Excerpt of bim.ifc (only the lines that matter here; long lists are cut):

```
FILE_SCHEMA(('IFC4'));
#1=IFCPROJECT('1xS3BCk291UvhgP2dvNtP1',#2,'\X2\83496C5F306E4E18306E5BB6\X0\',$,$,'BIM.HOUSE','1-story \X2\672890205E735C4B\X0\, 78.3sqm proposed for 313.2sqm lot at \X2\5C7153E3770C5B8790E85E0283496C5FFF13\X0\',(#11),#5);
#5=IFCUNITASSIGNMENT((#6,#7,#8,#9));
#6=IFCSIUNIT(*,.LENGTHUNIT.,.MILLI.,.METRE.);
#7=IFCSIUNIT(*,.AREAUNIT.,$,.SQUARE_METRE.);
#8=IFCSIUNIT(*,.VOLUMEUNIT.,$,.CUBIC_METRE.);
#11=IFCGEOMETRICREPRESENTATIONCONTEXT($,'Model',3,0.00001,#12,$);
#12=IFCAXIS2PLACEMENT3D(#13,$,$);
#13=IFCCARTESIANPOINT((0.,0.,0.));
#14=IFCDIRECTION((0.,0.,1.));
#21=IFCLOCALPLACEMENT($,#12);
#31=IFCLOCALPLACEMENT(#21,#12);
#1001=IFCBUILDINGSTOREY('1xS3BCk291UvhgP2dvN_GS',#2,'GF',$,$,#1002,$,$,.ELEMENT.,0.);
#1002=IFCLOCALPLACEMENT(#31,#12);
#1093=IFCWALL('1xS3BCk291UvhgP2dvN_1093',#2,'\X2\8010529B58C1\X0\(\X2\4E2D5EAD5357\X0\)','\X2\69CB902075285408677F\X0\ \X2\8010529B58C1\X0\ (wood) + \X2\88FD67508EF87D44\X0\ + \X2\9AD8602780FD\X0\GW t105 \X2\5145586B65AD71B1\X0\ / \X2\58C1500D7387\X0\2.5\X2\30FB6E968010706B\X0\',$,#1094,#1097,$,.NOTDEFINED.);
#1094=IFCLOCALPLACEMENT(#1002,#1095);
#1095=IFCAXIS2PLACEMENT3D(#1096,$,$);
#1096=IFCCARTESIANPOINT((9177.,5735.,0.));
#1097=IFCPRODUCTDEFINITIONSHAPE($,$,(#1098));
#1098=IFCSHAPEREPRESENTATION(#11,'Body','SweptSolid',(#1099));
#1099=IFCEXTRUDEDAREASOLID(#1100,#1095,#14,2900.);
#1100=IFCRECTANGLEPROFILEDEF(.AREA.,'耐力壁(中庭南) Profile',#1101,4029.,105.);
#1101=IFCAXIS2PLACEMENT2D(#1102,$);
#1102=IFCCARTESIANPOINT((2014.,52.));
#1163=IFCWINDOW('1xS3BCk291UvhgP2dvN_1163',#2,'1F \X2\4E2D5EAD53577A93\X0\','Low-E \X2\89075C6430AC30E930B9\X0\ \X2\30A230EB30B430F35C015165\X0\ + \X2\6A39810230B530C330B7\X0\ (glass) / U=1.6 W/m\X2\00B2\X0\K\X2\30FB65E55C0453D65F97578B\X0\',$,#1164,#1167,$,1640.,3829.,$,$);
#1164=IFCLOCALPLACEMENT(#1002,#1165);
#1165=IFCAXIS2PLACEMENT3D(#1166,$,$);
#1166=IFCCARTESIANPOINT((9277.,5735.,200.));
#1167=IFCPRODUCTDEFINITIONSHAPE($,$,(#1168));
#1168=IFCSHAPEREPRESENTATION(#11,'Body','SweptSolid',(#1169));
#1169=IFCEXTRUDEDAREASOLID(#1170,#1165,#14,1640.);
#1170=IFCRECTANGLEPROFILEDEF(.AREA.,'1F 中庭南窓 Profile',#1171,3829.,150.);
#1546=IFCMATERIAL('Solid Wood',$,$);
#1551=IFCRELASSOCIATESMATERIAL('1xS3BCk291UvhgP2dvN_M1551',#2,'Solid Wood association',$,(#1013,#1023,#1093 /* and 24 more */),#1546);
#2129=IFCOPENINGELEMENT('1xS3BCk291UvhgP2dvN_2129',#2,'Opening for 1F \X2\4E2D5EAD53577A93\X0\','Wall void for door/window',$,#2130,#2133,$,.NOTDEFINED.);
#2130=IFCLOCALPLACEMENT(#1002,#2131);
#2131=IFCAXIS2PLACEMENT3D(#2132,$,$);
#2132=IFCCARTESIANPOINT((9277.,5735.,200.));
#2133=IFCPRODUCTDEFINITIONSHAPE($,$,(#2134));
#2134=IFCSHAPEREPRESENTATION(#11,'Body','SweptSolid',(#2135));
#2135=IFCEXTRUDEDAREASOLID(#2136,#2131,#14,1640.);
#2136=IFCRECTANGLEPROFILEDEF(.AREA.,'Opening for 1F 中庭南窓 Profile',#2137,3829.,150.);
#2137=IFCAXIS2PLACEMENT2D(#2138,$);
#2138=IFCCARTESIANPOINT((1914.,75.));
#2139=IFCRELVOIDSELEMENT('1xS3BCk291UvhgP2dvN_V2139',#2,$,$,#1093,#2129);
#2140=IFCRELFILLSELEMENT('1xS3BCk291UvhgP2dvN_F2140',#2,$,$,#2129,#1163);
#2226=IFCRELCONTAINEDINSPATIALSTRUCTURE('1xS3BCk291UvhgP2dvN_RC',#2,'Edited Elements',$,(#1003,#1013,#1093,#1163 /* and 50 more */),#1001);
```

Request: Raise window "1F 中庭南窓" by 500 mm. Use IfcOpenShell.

```python
import numpy as np
import ifcopenshell
import ifcopenshell.api.geometry
import ifcopenshell.util.placement
import ifcopenshell.util.unit

model = ifcopenshell.open("bim.ifc")
unit_scale = ifcopenshell.util.unit.calculate_unit_scale(model)

window = model.by_guid("1xS3BCk291UvhgP2dvN_1163")
opening = window.FillsVoids[0].RelatingOpeningElement
dz = 0.5 / unit_scale

shift = np.array([0.0, 0.0, dz])
# The window is not placed relative to its opening, so move both.
for product in (opening, window):
    matrix = ifcopenshell.util.placement.get_local_placement(product.ObjectPlacement)
    matrix[:3, 3] += shift
    ifcopenshell.api.geometry.edit_object_placement(model, product=product, matrix=matrix, is_si=False)

print(f"moved by {dz * unit_scale:+.3f} m")

model.write("bim_rev.ifc")
```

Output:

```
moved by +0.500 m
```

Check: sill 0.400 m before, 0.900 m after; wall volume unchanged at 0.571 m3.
